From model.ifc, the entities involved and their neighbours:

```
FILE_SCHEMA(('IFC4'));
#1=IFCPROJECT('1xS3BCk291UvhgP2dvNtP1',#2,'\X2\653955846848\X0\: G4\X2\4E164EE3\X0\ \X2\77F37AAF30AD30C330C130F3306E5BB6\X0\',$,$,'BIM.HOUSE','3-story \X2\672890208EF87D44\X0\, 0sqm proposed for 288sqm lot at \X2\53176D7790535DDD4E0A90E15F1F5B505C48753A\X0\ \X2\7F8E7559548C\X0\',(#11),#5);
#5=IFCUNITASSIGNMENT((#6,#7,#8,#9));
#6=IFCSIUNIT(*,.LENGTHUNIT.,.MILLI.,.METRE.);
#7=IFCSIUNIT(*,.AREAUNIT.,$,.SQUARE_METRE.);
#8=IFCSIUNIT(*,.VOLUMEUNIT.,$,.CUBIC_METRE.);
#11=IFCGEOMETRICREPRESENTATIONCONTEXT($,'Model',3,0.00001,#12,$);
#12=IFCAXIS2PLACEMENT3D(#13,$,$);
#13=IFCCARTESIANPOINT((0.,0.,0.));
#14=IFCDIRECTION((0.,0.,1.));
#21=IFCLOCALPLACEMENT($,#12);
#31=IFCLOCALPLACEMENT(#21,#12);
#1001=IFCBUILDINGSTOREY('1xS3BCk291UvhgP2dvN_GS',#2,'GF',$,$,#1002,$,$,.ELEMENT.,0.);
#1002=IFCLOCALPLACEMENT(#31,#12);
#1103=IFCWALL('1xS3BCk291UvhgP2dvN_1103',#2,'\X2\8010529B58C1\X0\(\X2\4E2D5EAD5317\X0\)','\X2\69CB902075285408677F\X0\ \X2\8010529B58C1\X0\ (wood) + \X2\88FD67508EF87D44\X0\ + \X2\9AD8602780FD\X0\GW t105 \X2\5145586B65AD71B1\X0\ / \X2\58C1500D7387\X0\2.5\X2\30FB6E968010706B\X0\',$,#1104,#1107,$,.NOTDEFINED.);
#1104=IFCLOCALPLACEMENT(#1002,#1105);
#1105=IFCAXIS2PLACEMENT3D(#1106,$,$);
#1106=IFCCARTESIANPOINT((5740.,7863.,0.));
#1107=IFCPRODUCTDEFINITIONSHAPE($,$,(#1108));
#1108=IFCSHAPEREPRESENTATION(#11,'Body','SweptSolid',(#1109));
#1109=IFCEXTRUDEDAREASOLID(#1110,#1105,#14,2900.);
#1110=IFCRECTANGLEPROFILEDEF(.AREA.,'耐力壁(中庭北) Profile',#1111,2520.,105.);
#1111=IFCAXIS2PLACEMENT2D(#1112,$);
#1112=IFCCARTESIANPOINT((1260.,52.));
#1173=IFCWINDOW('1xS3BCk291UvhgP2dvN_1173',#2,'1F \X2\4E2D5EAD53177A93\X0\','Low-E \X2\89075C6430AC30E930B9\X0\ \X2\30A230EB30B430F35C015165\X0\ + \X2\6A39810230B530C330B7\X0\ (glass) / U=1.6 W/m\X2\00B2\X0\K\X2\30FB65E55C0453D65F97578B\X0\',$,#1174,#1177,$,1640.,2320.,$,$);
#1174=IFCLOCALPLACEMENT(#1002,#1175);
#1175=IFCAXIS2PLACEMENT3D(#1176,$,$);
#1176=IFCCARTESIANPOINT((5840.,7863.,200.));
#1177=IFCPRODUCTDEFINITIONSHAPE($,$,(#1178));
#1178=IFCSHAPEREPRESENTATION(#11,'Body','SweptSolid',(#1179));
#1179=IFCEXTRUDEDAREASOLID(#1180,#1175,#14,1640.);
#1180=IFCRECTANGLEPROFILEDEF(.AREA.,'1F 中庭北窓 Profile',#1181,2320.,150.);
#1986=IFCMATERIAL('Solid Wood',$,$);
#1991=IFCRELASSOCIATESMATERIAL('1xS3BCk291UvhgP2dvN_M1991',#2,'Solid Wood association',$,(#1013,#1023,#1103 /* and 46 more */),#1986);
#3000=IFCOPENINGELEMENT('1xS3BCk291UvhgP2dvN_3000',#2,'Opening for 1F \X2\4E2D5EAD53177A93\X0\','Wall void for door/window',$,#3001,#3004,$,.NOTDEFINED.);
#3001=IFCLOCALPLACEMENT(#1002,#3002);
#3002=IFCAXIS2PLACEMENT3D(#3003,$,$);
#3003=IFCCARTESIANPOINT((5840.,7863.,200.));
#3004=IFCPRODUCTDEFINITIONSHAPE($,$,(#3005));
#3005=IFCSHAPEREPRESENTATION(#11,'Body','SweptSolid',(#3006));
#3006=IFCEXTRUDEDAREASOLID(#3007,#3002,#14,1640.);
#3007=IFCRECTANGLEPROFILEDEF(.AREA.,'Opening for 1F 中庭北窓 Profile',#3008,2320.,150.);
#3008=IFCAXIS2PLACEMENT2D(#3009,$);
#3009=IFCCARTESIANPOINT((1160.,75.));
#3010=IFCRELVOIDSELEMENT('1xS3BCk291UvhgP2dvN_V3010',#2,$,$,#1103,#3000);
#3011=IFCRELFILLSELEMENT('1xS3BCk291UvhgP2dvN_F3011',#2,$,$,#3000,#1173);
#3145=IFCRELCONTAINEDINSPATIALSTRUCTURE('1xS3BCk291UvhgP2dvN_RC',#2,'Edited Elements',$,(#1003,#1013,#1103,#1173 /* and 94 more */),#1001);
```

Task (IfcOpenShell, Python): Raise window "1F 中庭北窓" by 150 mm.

```python
import numpy as np
import ifcopenshell
import ifcopenshell.api.geometry
import ifcopenshell.util.placement
import ifcopenshell.util.unit

model = ifcopenshell.open("model.ifc")
unit_scale = ifcopenshell.util.unit.calculate_unit_scale(model)

window = model.by_guid("1xS3BCk291UvhgP2dvN_1173")
opening = window.FillsVoids[0].RelatingOpeningElement
dz = 0.15 / unit_scale

shift = np.array([0.0, 0.0, dz])
# The window is not placed relative to its opening, so move both.
for product in (opening, window):
    matrix = ifcopenshell.util.placement.get_local_placement(product.ObjectPlacement)
    matrix[:3, 3] += shift
    ifcopenshell.api.geometry.edit_object_placement(model, product=product, matrix=matrix, is_si=False)

print(f"moved by {dz * unit_scale:+.3f} m")

model.write("model_rev.ifc")
```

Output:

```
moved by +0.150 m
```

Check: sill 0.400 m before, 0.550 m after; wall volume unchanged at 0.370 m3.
